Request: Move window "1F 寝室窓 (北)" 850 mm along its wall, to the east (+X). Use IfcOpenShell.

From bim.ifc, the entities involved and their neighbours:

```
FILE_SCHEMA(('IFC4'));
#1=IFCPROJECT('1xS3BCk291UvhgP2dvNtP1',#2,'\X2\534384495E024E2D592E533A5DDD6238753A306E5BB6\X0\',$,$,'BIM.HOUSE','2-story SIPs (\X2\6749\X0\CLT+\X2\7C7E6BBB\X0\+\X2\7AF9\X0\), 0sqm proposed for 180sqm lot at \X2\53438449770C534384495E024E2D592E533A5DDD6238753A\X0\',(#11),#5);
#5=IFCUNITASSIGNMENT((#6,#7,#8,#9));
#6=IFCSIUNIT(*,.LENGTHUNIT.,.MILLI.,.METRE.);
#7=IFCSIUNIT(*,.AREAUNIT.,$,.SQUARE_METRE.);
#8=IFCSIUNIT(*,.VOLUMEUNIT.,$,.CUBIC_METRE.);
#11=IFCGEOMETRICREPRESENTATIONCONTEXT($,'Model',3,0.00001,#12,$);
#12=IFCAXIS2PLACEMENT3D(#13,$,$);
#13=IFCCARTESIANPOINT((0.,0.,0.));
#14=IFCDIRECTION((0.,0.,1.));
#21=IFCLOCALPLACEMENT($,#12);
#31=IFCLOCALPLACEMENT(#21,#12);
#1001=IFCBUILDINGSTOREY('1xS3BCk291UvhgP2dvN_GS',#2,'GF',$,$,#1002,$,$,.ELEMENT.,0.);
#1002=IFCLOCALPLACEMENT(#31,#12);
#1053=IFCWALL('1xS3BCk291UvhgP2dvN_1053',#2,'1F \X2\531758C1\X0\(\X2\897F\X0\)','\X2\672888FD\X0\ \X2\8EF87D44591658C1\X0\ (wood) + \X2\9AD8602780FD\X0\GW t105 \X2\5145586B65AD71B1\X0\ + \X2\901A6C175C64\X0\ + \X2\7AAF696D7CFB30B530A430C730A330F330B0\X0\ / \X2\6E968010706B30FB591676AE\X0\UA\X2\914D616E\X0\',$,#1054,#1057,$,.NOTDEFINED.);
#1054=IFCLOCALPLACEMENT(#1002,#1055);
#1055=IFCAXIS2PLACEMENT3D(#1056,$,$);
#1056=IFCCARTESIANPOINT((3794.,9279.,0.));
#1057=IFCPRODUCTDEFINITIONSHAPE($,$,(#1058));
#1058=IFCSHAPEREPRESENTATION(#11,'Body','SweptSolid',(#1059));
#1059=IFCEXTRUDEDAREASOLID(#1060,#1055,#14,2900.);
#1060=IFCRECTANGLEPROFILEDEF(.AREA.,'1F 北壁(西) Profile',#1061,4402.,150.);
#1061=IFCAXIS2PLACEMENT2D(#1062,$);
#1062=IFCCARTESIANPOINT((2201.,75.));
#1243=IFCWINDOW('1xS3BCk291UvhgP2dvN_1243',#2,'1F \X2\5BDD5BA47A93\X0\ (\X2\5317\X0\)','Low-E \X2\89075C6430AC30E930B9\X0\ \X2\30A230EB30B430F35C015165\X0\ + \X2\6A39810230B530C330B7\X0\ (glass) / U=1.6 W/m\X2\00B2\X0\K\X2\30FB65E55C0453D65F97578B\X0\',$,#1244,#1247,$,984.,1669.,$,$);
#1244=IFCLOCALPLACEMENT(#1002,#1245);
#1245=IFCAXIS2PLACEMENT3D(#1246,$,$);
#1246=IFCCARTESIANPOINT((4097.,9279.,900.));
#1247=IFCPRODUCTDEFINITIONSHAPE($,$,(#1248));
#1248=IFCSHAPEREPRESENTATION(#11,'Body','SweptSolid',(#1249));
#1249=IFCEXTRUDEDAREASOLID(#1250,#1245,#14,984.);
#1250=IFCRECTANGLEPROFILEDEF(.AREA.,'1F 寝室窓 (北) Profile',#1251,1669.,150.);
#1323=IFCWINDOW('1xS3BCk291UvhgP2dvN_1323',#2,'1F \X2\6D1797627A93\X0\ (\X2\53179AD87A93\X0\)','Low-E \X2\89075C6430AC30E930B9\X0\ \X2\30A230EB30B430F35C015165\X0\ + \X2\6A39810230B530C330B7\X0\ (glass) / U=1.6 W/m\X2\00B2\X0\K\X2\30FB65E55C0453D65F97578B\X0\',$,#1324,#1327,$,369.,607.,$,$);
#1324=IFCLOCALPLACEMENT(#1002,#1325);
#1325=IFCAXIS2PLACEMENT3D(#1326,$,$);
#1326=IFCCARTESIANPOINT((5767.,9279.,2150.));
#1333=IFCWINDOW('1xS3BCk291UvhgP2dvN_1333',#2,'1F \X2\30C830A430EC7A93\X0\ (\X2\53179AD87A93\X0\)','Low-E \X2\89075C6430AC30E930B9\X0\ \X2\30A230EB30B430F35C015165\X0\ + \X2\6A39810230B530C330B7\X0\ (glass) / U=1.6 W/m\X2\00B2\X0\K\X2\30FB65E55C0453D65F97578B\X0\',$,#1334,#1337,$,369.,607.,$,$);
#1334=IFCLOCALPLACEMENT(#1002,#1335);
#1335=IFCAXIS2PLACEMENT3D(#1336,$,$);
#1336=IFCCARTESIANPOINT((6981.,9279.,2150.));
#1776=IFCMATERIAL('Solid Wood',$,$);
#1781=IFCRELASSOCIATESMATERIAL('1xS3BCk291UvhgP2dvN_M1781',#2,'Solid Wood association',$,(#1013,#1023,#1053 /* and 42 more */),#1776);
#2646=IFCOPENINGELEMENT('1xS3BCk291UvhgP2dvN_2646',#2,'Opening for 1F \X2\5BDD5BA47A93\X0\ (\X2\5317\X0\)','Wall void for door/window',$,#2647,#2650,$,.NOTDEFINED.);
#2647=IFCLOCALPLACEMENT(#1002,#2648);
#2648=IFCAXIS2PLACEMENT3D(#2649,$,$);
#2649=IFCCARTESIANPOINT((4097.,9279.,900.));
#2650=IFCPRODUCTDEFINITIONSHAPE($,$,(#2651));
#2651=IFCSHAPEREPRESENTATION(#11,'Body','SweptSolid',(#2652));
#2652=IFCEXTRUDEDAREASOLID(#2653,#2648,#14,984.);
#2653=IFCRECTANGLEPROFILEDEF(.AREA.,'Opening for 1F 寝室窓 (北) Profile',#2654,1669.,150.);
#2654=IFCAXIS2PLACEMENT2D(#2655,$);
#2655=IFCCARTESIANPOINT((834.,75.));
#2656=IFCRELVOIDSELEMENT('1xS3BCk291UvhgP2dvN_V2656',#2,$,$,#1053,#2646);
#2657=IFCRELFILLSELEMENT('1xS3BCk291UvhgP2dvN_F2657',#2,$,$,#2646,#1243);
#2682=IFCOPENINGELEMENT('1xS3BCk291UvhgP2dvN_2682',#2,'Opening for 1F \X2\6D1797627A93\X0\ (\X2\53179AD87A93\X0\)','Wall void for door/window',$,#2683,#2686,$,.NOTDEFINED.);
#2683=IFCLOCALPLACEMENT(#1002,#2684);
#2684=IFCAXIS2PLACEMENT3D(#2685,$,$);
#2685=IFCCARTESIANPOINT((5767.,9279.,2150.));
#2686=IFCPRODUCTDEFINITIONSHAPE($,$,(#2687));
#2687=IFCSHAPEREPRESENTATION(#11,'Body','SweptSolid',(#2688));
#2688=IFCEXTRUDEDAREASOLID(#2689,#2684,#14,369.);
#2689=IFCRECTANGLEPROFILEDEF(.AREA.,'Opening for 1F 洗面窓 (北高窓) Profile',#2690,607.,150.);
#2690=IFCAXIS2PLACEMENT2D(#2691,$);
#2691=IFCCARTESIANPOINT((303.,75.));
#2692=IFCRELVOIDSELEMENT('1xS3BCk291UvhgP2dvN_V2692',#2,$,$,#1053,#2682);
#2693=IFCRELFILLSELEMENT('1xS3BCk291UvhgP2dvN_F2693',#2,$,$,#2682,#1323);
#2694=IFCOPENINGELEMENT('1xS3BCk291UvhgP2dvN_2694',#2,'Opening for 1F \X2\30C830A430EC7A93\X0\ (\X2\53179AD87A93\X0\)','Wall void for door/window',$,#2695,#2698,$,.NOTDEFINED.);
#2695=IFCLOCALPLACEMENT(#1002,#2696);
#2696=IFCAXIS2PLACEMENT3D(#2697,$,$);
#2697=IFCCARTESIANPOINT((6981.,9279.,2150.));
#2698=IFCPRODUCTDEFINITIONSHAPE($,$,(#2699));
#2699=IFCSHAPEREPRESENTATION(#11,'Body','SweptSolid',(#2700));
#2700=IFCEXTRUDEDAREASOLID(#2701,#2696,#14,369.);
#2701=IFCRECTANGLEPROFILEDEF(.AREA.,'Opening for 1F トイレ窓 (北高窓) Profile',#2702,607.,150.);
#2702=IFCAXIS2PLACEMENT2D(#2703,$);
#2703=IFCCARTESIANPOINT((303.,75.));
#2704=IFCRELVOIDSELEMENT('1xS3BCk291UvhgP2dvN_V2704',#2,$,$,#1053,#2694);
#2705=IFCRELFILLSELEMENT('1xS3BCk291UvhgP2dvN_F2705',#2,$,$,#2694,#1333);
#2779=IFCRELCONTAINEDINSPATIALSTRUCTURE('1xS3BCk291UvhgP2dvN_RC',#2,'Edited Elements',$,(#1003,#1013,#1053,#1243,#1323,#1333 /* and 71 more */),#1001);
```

```python
import ifcopenshell
import ifcopenshell.api.geometry
import ifcopenshell.util.placement

model = ifcopenshell.open("bim.ifc")

window = model.by_guid("1xS3BCk291UvhgP2dvN_1243")
opening = window.FillsVoids[0].RelatingOpeningElement
wall = opening.VoidsElements[0].RelatingBuildingElement

wall_matrix = ifcopenshell.util.placement.get_local_placement(wall.ObjectPlacement)
shift = wall_matrix[:3, 0] * 850.0
before = ifcopenshell.util.placement.get_local_placement(window.ObjectPlacement)[:3, 3].copy()

# The window is not placed relative to its opening, so move both.
for product in (opening, window):
    matrix = ifcopenshell.util.placement.get_local_placement(product.ObjectPlacement)
    matrix[:3, 3] += shift
    ifcopenshell.api.geometry.edit_object_placement(model, product=product, matrix=matrix, is_si=False)

after = ifcopenshell.util.placement.get_local_placement(window.ObjectPlacement)[:3, 3]
print("window moved by", (after - before).round(3) + 0.0)

model.write("bim_updated.ifc")
```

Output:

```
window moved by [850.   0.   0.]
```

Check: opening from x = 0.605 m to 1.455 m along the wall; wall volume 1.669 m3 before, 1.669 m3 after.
